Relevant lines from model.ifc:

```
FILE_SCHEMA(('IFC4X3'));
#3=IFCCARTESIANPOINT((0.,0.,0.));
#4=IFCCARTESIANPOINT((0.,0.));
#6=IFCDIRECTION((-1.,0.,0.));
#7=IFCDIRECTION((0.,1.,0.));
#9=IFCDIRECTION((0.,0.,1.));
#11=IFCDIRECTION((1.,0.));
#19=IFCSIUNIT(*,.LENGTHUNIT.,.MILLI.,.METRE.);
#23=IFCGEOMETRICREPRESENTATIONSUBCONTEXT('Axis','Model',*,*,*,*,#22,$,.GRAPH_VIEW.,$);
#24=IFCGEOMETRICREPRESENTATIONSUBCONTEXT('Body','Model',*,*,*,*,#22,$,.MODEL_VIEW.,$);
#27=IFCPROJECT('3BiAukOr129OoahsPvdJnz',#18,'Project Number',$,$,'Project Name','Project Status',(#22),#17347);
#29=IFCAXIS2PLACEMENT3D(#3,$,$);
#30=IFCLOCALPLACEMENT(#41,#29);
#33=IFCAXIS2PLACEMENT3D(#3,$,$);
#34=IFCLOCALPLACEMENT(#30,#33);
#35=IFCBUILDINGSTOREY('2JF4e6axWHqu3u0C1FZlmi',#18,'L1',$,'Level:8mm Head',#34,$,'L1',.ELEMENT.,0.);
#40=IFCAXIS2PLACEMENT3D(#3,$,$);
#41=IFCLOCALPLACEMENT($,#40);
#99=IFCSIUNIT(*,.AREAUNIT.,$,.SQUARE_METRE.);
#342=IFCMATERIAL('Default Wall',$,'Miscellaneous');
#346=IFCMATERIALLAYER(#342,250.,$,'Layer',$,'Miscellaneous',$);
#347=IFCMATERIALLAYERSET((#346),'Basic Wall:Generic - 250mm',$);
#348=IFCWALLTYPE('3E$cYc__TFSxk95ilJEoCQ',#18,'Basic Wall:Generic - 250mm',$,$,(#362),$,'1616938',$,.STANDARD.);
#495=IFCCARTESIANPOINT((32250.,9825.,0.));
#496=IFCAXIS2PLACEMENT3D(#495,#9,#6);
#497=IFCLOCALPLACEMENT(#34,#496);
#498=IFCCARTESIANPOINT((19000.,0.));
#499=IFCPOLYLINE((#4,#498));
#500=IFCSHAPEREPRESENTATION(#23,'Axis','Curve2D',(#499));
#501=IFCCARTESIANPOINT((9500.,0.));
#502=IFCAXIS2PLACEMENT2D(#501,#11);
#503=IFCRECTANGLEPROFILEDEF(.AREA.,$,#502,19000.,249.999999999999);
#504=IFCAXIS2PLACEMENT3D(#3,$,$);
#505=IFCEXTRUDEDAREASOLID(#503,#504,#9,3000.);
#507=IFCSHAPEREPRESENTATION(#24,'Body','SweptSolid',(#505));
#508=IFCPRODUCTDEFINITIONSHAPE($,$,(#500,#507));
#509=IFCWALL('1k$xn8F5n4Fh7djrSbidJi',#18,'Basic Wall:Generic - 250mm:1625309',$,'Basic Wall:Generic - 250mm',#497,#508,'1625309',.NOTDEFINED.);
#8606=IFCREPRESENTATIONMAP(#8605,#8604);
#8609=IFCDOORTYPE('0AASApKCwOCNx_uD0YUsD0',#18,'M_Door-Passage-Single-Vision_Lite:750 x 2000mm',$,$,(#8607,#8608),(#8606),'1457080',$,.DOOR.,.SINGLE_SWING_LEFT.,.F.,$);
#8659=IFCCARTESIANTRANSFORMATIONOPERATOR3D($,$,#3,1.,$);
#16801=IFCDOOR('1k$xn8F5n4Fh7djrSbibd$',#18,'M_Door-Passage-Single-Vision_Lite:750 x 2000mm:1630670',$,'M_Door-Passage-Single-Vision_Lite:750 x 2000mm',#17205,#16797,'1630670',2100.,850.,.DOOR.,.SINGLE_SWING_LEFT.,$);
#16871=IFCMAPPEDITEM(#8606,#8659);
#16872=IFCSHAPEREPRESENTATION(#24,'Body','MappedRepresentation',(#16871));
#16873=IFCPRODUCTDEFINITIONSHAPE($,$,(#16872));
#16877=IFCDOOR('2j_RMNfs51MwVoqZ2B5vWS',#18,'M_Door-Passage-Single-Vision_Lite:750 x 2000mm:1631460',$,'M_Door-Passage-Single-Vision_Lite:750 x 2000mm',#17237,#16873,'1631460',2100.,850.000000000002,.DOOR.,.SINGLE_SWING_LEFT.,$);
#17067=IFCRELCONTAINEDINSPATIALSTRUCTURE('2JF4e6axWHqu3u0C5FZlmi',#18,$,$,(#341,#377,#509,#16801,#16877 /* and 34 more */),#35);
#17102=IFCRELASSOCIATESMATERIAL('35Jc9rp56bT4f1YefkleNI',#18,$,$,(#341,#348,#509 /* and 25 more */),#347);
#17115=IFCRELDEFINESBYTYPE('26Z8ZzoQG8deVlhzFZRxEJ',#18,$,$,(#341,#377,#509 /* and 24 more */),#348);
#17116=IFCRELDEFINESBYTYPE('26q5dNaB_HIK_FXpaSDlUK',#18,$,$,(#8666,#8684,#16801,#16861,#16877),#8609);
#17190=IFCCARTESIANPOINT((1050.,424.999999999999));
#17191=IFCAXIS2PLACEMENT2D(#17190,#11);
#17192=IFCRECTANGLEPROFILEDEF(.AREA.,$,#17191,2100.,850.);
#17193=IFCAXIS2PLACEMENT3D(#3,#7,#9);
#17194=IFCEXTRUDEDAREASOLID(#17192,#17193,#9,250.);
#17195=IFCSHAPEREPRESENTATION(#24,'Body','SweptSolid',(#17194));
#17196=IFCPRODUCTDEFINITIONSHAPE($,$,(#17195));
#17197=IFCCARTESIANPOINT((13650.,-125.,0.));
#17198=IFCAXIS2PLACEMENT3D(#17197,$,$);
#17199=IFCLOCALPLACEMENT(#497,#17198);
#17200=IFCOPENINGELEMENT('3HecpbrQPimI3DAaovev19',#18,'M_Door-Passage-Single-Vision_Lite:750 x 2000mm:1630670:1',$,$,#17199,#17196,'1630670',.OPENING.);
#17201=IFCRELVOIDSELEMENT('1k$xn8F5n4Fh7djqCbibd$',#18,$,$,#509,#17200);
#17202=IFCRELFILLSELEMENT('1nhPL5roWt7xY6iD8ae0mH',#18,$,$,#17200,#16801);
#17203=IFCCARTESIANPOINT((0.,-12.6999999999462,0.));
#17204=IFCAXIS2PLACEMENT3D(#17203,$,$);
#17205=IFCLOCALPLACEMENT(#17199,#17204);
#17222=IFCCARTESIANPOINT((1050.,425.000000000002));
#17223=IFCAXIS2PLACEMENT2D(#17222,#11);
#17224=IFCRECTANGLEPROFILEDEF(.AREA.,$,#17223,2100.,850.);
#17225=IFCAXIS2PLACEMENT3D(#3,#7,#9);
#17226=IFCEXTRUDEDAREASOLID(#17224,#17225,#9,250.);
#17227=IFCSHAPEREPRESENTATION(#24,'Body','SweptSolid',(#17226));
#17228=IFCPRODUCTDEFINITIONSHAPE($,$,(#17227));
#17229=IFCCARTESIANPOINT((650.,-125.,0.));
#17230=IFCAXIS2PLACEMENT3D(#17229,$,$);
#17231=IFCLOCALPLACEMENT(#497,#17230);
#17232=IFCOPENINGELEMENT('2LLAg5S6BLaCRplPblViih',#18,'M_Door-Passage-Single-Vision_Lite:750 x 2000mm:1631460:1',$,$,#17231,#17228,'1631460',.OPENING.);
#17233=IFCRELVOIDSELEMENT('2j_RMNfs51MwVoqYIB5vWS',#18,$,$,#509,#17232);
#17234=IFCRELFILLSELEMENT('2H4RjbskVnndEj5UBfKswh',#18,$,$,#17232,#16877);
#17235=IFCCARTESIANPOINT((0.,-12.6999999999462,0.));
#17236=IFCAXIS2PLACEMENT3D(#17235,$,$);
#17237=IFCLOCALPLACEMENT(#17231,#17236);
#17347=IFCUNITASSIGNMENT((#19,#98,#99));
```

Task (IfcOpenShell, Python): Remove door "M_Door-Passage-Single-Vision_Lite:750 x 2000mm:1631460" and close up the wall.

```python
import ifcopenshell
import ifcopenshell.api.feature
import ifcopenshell.api.root
import ifcopenshell.geom
import ifcopenshell.util.shape

model = ifcopenshell.open("model.ifc")
settings = ifcopenshell.geom.settings()


def volume(element):
    """Net volume in cubic metres, openings subtracted."""
    shape = ifcopenshell.geom.create_shape(settings, element)
    return ifcopenshell.util.shape.get_volume(shape.geometry)


door = model.by_guid("2j_RMNfs51MwVoqZ2B5vWS")
opening = door.FillsVoids[0].RelatingOpeningElement
wall = opening.VoidsElements[0].RelatingBuildingElement
before = volume(wall)

ifcopenshell.api.root.remove_product(model, product=door)
ifcopenshell.api.feature.remove_feature(model, feature=opening)

after = volume(wall)

print(f"wall volume {before:.3f} -> {after:.3f} m3")

model.write("model_updated.ifc")
```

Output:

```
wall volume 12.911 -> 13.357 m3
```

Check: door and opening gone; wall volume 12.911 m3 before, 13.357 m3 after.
